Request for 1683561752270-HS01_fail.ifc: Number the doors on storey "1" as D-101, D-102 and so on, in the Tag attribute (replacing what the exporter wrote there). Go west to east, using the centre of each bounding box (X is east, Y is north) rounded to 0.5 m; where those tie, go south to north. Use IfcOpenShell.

First a look at what the model holds.

```python
import ifcopenshell
import ifcopenshell.util.element
import ifcopenshell.util.placement

model = ifcopenshell.open("1683561752270-HS01_fail.ifc")
print(model.schema)
storey = next(s for s in model.by_type("IfcBuildingStorey") if s.Name == "1")
doors = [e for e in ifcopenshell.util.element.get_decomposition(storey) if e.is_a("IfcDoor")]
for e in sorted(doors, key=lambda e: e.id()):
    origin = ifcopenshell.util.placement.get_local_placement(e.ObjectPlacement)[:3, 3]
    print(e.id(), e.Tag, e.Name, origin.round(2) + 0.0, sep=" | ")
```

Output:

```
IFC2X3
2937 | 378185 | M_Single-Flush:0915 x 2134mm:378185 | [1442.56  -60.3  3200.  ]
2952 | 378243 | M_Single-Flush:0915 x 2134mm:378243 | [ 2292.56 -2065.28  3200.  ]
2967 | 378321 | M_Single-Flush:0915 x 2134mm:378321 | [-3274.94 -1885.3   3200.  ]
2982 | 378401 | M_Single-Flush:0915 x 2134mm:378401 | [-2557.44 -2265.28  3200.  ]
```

```python
import ifcopenshell
import ifcopenshell.geom
import ifcopenshell.util.element
import ifcopenshell.util.shape

model = ifcopenshell.open("1683561752270-HS01_fail.ifc")
settings = ifcopenshell.geom.settings()
settings.set("use-world-coords", True)


def centre(element):
    shape = ifcopenshell.geom.create_shape(settings, element)
    return ifcopenshell.util.shape.get_bbox_centroid(shape.geometry)


storey = next(s for s in model.by_type("IfcBuildingStorey") if s.Name == "1")
doors = [e for e in ifcopenshell.util.element.get_decomposition(storey) if e.is_a("IfcDoor")]

# Insertion points can sit at a corner or the storey origin, so sort by the geometry (in metres).
centres = {e: centre(e) for e in doors}
doors.sort(key=lambda e: (round(centres[e][0] / 0.5), centres[e][1]))

for i, e in enumerate(doors, start=1):
    number = f"D-1{i:02d}"
    e.Tag = number
    print(e.id(), number)

model.write("1683561752270-HS01_fail_v2.ifc")
```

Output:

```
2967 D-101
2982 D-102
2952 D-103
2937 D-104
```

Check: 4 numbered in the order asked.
